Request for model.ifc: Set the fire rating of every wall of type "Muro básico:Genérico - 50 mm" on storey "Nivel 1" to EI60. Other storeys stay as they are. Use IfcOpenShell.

First a look at what the model holds.

```python
import ifcopenshell
import ifcopenshell.util.element

model = ifcopenshell.open("model.ifc")
print(model.schema)
storey = next(s for s in model.by_type("IfcBuildingStorey") if s.Name == "Nivel 1")
walls = [e for e in ifcopenshell.util.element.get_decomposition(storey) if e.is_a("IfcWall")]
seen = {}
for e in walls:
    element_type = ifcopenshell.util.element.get_type(e)
    key = (element_type.Name if element_type != e and element_type else None, ifcopenshell.util.element.get_pset(e, "Pset_WallCommon", "FireRating"))
    seen[key] = seen.get(key, 0) + 1
for (name, value), count in sorted(seen.items(), key=str):
    print(count, "x", name, "|", value)
```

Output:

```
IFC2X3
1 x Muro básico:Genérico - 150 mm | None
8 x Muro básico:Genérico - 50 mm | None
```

```python
import ifcopenshell
import ifcopenshell.api.pset
import ifcopenshell.util.element

model = ifcopenshell.open("model.ifc")

storey = next(s for s in model.by_type("IfcBuildingStorey") if s.Name == "Nivel 1")
walls = [e for e in ifcopenshell.util.element.get_decomposition(storey) if e.is_a("IfcWall")]

count = 0
for e in walls:
    element_type = ifcopenshell.util.element.get_type(e)
    if element_type in (None, e) or element_type.Name != "Muro básico:Genérico - 50 mm":
        continue
    # add_pset returns the element's existing set when there is one.
    pset = ifcopenshell.api.pset.add_pset(model, product=e, name="Pset_WallCommon")
    ifcopenshell.api.pset.edit_pset(model, pset=pset, properties={"FireRating": "EI60"})
    count += 1

print(count, "walls updated")

model.write("model_rev.ifc")
```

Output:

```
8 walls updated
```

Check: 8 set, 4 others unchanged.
